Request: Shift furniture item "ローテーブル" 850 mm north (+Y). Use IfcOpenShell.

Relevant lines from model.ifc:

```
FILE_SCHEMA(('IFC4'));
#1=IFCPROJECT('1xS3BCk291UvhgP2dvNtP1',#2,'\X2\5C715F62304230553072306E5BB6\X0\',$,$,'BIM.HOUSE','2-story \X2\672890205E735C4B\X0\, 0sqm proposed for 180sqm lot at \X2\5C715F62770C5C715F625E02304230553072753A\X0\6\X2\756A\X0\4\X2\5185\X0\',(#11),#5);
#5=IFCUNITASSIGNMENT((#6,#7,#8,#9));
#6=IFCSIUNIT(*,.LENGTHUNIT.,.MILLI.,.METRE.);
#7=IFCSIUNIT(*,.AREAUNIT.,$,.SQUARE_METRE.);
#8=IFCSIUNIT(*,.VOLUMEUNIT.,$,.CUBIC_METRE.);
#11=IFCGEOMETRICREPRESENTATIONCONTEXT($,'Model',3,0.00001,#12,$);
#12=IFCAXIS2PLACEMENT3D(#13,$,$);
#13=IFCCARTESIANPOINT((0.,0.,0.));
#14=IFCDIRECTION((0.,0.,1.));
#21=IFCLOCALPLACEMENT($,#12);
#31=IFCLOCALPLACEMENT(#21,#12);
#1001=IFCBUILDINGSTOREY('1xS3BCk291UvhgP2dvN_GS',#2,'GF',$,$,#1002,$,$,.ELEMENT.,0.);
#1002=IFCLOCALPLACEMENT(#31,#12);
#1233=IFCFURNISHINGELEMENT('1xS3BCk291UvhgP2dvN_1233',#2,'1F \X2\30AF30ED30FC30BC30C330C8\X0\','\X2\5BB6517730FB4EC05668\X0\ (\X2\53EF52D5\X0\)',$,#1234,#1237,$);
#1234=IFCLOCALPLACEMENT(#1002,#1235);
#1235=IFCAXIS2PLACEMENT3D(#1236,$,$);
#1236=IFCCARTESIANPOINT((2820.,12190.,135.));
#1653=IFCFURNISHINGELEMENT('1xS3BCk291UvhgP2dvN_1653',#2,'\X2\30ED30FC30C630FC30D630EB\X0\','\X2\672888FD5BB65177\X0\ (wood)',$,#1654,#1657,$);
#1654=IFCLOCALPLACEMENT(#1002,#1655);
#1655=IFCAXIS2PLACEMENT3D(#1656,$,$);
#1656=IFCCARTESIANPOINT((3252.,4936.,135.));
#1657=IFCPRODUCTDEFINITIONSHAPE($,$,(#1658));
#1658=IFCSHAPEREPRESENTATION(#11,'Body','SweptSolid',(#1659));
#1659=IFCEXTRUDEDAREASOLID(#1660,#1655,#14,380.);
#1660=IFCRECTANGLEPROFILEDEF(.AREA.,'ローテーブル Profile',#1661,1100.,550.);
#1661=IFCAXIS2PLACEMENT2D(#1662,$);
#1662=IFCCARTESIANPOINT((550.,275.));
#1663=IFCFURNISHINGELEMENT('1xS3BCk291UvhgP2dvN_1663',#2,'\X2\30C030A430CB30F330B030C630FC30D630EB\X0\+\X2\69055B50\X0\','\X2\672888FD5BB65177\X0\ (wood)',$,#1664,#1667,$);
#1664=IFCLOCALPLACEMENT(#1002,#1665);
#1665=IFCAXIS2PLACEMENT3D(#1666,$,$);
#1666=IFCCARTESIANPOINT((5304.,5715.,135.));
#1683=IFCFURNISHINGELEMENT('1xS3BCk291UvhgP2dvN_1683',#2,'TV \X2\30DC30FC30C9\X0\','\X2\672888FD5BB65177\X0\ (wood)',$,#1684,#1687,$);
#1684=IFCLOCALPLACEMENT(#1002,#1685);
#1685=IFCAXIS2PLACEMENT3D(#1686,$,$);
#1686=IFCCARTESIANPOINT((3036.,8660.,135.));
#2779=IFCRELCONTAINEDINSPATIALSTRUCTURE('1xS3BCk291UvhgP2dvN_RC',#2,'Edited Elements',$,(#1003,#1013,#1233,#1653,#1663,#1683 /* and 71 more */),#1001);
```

```python
import ifcopenshell
import ifcopenshell.api.geometry
import ifcopenshell.util.placement
import ifcopenshell.util.unit

model = ifcopenshell.open("model.ifc")
unit_scale = ifcopenshell.util.unit.calculate_unit_scale(model)

item = model.by_id(1653)
matrix = ifcopenshell.util.placement.get_local_placement(item.ObjectPlacement)
matrix[1, 3] += 0.85 / unit_scale
ifcopenshell.api.geometry.edit_object_placement(model, product=item, matrix=matrix, is_si=False)

print(ifcopenshell.util.placement.get_local_placement(item.ObjectPlacement).round(3) + 0.0)

model.write("model_rev.ifc")
```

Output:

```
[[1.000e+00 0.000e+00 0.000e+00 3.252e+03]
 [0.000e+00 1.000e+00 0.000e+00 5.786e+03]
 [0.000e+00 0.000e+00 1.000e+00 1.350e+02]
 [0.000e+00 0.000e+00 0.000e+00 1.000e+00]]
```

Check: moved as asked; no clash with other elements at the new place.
